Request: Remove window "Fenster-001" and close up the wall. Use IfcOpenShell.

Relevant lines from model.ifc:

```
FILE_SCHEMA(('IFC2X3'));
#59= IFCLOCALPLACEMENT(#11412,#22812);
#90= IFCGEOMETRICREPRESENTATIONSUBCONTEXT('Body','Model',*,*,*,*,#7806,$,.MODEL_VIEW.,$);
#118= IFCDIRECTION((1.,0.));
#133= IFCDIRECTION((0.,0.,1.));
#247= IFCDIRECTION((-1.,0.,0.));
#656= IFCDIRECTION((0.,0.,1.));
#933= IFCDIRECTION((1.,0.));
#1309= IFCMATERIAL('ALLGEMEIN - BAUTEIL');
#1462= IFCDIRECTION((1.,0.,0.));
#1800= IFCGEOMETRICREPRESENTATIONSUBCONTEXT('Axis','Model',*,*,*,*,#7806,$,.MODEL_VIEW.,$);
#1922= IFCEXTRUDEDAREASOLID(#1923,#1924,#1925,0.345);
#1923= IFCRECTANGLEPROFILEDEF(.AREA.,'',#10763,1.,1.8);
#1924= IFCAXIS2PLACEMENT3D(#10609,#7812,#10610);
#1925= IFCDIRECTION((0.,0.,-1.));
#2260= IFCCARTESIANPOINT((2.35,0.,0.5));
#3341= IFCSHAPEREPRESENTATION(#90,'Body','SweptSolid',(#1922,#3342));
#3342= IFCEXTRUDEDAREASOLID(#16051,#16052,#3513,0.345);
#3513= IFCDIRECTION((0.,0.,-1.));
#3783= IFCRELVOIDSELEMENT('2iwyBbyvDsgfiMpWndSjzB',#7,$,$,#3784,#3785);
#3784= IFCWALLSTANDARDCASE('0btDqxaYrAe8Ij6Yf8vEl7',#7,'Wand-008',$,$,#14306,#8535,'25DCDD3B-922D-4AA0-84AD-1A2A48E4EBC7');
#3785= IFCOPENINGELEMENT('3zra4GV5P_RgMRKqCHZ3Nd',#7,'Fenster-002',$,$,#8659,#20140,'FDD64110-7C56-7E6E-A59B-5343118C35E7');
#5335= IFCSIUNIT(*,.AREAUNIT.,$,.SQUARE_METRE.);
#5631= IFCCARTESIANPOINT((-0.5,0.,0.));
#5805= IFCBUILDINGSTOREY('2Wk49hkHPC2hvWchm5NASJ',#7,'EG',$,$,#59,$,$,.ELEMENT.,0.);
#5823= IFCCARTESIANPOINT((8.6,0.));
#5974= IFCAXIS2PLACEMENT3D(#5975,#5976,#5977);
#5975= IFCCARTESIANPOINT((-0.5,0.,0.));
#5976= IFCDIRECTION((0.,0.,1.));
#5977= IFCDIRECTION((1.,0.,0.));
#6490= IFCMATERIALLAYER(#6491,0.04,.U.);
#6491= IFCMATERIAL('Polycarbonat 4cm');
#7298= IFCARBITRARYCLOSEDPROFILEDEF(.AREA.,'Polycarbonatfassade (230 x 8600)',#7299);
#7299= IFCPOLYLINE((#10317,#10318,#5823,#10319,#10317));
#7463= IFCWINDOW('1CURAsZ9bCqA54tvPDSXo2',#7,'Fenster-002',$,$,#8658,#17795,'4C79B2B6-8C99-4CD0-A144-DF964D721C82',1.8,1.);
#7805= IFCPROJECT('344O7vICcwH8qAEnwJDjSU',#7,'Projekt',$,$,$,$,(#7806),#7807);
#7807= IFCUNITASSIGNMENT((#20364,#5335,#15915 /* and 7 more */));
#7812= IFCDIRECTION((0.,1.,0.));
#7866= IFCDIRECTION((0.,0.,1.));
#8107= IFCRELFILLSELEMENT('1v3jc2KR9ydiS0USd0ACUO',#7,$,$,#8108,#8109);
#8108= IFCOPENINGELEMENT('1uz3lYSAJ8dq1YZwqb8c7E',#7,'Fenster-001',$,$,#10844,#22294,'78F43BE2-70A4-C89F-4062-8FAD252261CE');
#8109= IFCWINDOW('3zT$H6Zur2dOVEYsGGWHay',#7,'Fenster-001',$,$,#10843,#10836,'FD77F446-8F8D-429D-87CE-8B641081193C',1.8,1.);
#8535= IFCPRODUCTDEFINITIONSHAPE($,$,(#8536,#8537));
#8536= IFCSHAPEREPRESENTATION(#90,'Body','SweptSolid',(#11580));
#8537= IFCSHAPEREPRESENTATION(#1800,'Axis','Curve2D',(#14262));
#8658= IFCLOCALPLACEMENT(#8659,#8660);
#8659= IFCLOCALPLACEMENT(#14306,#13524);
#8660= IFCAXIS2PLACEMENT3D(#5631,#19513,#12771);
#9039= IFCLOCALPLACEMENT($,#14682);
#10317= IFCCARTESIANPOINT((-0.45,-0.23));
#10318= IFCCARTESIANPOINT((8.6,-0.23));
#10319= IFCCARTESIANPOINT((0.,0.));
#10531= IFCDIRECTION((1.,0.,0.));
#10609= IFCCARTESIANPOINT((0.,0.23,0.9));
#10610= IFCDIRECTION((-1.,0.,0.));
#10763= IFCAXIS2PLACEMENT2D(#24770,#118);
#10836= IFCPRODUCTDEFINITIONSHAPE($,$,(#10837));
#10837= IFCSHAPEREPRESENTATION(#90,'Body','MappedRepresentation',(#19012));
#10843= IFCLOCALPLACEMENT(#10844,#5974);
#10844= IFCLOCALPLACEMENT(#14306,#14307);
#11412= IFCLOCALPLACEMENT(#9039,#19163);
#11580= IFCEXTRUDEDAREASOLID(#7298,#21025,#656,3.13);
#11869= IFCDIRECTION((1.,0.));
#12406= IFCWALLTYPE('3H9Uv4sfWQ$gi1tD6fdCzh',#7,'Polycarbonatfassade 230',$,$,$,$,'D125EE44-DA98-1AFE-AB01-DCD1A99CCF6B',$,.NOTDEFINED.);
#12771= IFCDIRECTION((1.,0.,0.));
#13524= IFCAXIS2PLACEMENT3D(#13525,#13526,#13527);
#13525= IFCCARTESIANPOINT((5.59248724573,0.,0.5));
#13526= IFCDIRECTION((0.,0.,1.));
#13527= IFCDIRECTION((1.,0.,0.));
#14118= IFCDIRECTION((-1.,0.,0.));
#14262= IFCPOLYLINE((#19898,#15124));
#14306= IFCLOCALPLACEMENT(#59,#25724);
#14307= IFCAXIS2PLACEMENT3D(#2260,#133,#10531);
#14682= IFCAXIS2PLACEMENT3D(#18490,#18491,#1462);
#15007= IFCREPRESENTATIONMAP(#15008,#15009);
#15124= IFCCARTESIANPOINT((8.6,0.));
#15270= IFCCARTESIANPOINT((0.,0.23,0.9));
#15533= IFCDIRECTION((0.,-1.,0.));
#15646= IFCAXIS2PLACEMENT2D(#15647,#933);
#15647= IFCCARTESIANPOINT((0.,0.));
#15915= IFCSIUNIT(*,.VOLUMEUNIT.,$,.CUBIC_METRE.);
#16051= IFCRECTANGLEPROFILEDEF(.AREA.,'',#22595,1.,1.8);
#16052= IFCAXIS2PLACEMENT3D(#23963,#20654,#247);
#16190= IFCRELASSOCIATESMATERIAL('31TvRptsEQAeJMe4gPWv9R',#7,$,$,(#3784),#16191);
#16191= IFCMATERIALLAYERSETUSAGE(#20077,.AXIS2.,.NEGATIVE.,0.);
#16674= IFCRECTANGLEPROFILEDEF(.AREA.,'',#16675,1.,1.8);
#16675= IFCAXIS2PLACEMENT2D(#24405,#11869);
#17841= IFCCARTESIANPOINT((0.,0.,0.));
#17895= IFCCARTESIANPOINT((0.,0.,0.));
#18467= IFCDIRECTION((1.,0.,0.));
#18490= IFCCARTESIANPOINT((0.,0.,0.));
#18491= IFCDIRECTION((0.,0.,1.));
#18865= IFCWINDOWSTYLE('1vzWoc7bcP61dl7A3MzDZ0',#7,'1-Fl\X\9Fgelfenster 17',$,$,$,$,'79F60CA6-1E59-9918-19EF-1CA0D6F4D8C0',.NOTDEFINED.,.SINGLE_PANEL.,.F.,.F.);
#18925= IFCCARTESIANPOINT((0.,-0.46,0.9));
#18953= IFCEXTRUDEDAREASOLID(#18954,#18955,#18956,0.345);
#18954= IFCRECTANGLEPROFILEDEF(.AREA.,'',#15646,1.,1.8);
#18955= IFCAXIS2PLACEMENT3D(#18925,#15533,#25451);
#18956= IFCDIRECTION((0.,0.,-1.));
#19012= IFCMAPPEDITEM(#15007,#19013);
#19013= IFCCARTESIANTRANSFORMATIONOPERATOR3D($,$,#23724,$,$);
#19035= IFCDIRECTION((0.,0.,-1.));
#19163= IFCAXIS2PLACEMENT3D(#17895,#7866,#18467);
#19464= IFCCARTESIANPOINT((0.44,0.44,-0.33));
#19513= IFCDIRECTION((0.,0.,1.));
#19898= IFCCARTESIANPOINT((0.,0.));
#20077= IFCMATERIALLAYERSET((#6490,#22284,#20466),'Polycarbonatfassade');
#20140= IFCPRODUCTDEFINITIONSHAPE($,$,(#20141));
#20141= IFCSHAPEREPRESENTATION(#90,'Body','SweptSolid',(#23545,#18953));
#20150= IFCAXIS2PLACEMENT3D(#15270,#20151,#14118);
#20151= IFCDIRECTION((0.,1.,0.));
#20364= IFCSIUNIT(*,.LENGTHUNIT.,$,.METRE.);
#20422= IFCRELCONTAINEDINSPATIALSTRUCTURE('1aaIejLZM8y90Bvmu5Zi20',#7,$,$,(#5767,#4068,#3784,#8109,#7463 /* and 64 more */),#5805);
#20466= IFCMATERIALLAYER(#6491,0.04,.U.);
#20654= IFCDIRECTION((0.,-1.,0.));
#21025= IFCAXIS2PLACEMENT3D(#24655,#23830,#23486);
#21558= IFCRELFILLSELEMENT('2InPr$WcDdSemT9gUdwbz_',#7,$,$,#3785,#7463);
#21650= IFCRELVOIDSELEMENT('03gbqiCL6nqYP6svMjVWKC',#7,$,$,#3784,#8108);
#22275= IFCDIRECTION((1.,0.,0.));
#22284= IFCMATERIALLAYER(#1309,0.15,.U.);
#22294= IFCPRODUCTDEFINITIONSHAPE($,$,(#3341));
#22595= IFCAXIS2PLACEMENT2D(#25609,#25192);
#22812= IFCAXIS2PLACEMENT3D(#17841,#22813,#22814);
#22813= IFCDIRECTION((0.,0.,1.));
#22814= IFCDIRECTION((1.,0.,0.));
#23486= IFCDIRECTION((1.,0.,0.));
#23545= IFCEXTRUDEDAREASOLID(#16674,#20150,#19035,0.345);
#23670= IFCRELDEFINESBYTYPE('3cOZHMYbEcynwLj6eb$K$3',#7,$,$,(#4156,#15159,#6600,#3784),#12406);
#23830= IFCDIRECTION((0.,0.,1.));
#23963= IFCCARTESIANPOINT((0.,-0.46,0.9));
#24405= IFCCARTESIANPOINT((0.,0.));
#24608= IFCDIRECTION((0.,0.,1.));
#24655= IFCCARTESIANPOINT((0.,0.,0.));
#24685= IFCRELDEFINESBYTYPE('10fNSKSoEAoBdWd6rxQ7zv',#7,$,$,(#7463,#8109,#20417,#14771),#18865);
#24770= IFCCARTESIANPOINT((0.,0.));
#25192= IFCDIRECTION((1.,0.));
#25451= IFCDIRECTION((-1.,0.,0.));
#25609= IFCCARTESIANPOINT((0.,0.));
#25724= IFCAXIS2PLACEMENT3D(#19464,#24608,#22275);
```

```python
import ifcopenshell
import ifcopenshell.api.feature
import ifcopenshell.api.root
import ifcopenshell.geom
import ifcopenshell.util.shape

model = ifcopenshell.open("model.ifc")
settings = ifcopenshell.geom.settings()


def volume(element):
    """Net volume in cubic metres, openings subtracted."""
    shape = ifcopenshell.geom.create_shape(settings, element)
    return ifcopenshell.util.shape.get_volume(shape.geometry)


window = model.by_id(8109)
opening = window.FillsVoids[0].RelatingOpeningElement
wall = opening.VoidsElements[0].RelatingBuildingElement
before = volume(wall)

ifcopenshell.api.root.remove_product(model, product=window)
ifcopenshell.api.feature.remove_feature(model, feature=opening)

after = volume(wall)

print(f"wall volume {before:.3f} -> {after:.3f} m3")

model.write("model_updated.ifc")
```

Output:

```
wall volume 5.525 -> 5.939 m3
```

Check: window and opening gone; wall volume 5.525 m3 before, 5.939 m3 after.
